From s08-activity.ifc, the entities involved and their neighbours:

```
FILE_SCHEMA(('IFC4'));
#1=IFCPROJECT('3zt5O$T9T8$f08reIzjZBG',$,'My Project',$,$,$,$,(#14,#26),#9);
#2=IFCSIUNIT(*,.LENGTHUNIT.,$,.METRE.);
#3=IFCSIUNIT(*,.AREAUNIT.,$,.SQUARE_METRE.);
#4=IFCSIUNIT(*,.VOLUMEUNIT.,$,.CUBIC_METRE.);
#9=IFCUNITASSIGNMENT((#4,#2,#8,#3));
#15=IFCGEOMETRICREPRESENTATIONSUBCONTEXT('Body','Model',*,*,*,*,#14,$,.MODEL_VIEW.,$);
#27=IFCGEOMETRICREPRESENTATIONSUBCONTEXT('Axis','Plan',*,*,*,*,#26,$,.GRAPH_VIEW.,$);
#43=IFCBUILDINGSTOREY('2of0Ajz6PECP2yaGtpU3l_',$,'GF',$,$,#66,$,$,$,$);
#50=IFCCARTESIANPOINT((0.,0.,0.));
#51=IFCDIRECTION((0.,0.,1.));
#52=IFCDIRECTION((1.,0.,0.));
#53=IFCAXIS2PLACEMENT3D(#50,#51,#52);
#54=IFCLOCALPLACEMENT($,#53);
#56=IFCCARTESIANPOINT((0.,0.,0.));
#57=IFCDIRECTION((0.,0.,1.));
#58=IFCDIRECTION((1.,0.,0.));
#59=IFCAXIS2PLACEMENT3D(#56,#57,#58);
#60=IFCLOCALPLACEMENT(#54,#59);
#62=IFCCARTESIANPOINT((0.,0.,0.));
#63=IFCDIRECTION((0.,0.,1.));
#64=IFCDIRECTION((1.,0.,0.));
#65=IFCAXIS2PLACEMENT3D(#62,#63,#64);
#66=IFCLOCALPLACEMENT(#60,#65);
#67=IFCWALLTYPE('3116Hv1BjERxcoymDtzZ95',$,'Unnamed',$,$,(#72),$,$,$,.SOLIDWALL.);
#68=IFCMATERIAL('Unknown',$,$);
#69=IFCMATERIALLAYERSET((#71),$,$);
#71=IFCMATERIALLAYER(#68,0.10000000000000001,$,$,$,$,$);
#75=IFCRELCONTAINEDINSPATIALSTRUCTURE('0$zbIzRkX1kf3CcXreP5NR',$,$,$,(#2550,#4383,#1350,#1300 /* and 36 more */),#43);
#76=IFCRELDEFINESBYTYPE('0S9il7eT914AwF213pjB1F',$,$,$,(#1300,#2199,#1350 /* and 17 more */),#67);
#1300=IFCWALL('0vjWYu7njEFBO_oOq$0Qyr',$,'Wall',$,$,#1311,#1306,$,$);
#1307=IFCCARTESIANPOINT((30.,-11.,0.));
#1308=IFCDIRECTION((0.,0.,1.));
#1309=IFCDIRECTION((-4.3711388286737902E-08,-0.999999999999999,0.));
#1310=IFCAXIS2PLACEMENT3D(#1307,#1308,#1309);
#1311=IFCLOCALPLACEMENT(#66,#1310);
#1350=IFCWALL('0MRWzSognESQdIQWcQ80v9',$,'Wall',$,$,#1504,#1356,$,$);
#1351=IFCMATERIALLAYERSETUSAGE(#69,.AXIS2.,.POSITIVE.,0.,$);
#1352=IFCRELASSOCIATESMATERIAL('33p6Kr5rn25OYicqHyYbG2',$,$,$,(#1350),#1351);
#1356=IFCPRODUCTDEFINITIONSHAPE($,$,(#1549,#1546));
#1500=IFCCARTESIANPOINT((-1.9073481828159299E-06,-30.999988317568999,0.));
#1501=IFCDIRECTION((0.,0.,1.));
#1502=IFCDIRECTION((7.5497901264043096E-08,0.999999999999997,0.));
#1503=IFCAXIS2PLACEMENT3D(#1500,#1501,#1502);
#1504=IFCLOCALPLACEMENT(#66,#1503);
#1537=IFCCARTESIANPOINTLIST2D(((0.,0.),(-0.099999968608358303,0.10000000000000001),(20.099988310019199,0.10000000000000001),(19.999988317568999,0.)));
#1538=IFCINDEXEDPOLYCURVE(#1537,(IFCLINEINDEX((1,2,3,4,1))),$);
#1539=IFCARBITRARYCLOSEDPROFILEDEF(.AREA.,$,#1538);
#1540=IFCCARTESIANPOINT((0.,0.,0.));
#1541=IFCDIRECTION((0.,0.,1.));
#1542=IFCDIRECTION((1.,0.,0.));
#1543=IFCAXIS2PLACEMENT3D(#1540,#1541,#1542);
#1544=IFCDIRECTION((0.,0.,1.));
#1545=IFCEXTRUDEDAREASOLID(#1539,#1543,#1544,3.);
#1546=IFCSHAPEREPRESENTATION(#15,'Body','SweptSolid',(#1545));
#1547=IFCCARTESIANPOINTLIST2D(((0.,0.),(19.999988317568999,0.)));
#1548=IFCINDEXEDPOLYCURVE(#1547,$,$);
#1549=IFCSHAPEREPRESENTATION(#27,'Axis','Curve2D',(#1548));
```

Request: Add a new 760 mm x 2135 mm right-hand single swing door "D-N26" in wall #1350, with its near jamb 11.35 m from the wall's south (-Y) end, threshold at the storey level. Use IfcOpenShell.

```python
import numpy as np
import ifcopenshell
import ifcopenshell.api.feature
import ifcopenshell.api.geometry
import ifcopenshell.api.root
import ifcopenshell.api.spatial
import ifcopenshell.geom
import ifcopenshell.util.element
import ifcopenshell.util.placement
import ifcopenshell.util.representation
import ifcopenshell.util.shape
import ifcopenshell.util.unit

model = ifcopenshell.open("s08-activity.ifc")
unit_scale = ifcopenshell.util.unit.calculate_unit_scale(model)
settings = ifcopenshell.geom.settings()


def volume(element):
    """Net volume in cubic metres, openings subtracted."""
    shape = ifcopenshell.geom.create_shape(settings, element)
    return ifcopenshell.util.shape.get_volume(shape.geometry)


wall = model.by_id(1350)
storey = ifcopenshell.util.element.get_container(wall, ifc_class="IfcBuildingStorey")
context = ifcopenshell.util.representation.get_context(model, "Model", "Body", "MODEL_VIEW")
before = volume(wall)

width, height, from_end, sill = 0.76, 2.135, 11.35, 0.0  # metres

# The wall runs along its own X axis, and the end named is its -X end.
wall_shape = ifcopenshell.geom.create_shape(settings, wall)
x, y, z = ifcopenshell.util.shape.get_vertices(wall_shape.geometry).T
start = x.min() + from_end
face, thickness = float(y.min()), float(y.max() - y.min())
wall_matrix = ifcopenshell.util.placement.get_local_placement(wall.ObjectPlacement)
level = ifcopenshell.util.placement.get_local_placement(storey.ObjectPlacement)[2, 3]


def in_wall(x, y):
    """Placement at x, y metres in the wall's axes, at sill height."""
    matrix = wall_matrix.copy()
    matrix[:, 3] = wall_matrix @ np.array([x / unit_scale, y / unit_scale, 0.0, 1.0])
    matrix[2, 3] = level + sill / unit_scale
    return matrix


# Opening: a box that overshoots both wall faces by 50 mm.
opening = ifcopenshell.api.root.create_entity(model, ifc_class="IfcOpeningElement", predefined_type="OPENING")
box = ifcopenshell.api.geometry.add_wall_representation(
    model, context=context, length=width, height=height, thickness=thickness + 0.1
)
ifcopenshell.api.geometry.assign_representation(model, product=opening, representation=box)
ifcopenshell.api.geometry.edit_object_placement(model, product=opening, matrix=in_wall(start, face - 0.05), is_si=False)
ifcopenshell.api.feature.add_feature(model, feature=opening, element=wall)

door = ifcopenshell.api.root.create_entity(model, ifc_class="IfcDoor", name="D-N26", predefined_type="DOOR")
door.OverallWidth, door.OverallHeight = width / unit_scale, height / unit_scale
door.OperationType = "SINGLE_SWING_RIGHT"
body = ifcopenshell.api.geometry.add_door_representation(
    model,
    context=context,
    overall_width=door.OverallWidth,
    overall_height=door.OverallHeight,
    operation_type="SINGLE_SWING_RIGHT",
    lining_properties={"LiningDepth": thickness / unit_scale, "ThresholdDepth": thickness / unit_scale},
)
ifcopenshell.api.geometry.assign_representation(model, product=door, representation=body)
ifcopenshell.api.spatial.assign_container(model, products=[door], relating_structure=storey)
ifcopenshell.api.feature.add_filling(model, opening=opening, element=door)

# The lining spans the wall, so the door starts at the wall face.
ifcopenshell.api.geometry.edit_object_placement(model, product=door, matrix=in_wall(start, face), is_si=False)

after = volume(wall)

print(f"wall volume {before:.3f} -> {after:.3f} m3")

model.write("s08-activity_updated.ifc")
```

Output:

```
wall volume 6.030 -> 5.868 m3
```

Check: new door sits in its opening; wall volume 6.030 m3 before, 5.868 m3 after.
